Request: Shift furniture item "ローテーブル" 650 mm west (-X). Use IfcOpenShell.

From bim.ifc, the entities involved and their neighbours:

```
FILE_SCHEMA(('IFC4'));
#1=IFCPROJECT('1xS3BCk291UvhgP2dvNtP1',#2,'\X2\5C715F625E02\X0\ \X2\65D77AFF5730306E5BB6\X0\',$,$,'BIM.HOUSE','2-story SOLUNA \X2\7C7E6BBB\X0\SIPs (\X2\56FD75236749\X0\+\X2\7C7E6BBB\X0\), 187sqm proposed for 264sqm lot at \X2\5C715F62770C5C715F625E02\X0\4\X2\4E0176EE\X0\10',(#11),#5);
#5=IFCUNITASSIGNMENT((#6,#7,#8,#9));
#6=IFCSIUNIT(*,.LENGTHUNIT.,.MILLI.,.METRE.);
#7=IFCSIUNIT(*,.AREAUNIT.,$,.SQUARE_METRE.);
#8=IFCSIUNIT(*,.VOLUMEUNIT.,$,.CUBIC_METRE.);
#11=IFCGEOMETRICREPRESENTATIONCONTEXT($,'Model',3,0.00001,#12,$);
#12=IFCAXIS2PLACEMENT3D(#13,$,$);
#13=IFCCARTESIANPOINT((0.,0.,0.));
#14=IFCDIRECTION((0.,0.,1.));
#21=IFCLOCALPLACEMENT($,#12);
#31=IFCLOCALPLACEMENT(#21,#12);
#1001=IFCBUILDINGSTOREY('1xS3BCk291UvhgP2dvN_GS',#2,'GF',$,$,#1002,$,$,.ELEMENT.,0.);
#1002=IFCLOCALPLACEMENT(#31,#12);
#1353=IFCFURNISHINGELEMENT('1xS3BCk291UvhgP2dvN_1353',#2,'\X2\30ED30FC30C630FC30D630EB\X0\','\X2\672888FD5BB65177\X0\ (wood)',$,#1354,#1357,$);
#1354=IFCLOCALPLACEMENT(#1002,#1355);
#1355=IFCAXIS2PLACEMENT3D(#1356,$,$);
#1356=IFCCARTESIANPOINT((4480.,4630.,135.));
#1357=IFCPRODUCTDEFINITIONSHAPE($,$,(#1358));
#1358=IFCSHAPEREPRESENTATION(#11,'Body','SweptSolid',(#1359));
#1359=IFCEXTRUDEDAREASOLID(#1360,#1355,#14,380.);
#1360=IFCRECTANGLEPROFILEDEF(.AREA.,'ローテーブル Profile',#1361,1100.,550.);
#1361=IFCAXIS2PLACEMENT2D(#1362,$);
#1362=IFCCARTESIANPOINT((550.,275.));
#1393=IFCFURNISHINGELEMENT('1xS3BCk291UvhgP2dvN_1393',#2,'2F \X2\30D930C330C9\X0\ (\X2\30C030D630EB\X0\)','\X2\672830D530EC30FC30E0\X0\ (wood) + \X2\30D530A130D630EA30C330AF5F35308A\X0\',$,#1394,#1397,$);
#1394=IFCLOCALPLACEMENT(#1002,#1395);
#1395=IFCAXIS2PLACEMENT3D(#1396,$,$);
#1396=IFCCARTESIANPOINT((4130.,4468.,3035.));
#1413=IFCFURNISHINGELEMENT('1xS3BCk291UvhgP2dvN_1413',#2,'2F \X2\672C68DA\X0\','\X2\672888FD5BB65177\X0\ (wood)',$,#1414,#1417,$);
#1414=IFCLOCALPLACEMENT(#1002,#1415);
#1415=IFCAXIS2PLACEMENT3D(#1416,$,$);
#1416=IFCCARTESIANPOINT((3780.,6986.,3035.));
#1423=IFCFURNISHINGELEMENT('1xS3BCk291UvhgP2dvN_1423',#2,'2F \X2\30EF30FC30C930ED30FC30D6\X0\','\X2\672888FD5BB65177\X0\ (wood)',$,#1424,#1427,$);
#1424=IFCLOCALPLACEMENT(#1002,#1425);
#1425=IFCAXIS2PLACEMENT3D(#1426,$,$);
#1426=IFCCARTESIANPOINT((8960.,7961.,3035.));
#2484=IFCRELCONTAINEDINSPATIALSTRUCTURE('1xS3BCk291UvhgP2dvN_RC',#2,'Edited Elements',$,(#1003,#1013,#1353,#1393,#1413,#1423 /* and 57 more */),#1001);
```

```python
import ifcopenshell
import ifcopenshell.api.geometry
import ifcopenshell.util.placement
import ifcopenshell.util.unit

model = ifcopenshell.open("bim.ifc")
unit_scale = ifcopenshell.util.unit.calculate_unit_scale(model)

item = model.by_id(1353)
matrix = ifcopenshell.util.placement.get_local_placement(item.ObjectPlacement)
matrix[0, 3] -= 0.65 / unit_scale
ifcopenshell.api.geometry.edit_object_placement(model, product=item, matrix=matrix, is_si=False)

print(ifcopenshell.util.placement.get_local_placement(item.ObjectPlacement).round(3) + 0.0)

model.write("bim-out.ifc")
```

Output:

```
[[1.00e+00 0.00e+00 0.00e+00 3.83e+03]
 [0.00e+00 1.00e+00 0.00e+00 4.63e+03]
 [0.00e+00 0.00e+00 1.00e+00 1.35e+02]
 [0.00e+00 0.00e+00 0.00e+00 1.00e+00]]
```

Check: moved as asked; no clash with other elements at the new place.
